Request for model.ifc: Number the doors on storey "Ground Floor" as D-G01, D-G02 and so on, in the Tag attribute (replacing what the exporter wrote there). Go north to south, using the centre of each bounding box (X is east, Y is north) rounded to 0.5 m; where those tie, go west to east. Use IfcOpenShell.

First a look at what the model holds.

```python
import ifcopenshell
import ifcopenshell.util.element
import ifcopenshell.util.placement

model = ifcopenshell.open("model.ifc")
print(model.schema)
storey = next(s for s in model.by_type("IfcBuildingStorey") if s.Name == "Ground Floor")
doors = [e for e in ifcopenshell.util.element.get_decomposition(storey) if e.is_a("IfcDoor")]
for e in sorted(doors, key=lambda e: e.id()):
    origin = ifcopenshell.util.placement.get_local_placement(e.ObjectPlacement)[:3, 3]
    print(e.id(), e.Tag, e.Name, origin.round(2) + 0.0, sep=" | ")
```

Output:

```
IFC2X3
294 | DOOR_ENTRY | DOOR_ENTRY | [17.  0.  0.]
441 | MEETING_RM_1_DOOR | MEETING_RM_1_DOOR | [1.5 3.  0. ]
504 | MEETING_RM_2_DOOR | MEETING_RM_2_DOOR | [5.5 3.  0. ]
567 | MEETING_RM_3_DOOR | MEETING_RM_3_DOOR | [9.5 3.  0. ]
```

```python
import ifcopenshell
import ifcopenshell.geom
import ifcopenshell.util.element
import ifcopenshell.util.shape

model = ifcopenshell.open("model.ifc")
settings = ifcopenshell.geom.settings()
settings.set("use-world-coords", True)


def centre(element):
    shape = ifcopenshell.geom.create_shape(settings, element)
    return ifcopenshell.util.shape.get_bbox_centroid(shape.geometry)


storey = next(s for s in model.by_type("IfcBuildingStorey") if s.Name == "Ground Floor")
doors = [e for e in ifcopenshell.util.element.get_decomposition(storey) if e.is_a("IfcDoor")]

# Insertion points can sit at a corner or the storey origin, so sort by the geometry (in metres).
centres = {e: centre(e) for e in doors}
doors.sort(key=lambda e: (-round(centres[e][1] / 0.5), centres[e][0]))

for i, e in enumerate(doors, start=1):
    number = f"D-G{i:02d}"
    e.Tag = number
    print(e.id(), number)

model.write("model_edited.ifc")
```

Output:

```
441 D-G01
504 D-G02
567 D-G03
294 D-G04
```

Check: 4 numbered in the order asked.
